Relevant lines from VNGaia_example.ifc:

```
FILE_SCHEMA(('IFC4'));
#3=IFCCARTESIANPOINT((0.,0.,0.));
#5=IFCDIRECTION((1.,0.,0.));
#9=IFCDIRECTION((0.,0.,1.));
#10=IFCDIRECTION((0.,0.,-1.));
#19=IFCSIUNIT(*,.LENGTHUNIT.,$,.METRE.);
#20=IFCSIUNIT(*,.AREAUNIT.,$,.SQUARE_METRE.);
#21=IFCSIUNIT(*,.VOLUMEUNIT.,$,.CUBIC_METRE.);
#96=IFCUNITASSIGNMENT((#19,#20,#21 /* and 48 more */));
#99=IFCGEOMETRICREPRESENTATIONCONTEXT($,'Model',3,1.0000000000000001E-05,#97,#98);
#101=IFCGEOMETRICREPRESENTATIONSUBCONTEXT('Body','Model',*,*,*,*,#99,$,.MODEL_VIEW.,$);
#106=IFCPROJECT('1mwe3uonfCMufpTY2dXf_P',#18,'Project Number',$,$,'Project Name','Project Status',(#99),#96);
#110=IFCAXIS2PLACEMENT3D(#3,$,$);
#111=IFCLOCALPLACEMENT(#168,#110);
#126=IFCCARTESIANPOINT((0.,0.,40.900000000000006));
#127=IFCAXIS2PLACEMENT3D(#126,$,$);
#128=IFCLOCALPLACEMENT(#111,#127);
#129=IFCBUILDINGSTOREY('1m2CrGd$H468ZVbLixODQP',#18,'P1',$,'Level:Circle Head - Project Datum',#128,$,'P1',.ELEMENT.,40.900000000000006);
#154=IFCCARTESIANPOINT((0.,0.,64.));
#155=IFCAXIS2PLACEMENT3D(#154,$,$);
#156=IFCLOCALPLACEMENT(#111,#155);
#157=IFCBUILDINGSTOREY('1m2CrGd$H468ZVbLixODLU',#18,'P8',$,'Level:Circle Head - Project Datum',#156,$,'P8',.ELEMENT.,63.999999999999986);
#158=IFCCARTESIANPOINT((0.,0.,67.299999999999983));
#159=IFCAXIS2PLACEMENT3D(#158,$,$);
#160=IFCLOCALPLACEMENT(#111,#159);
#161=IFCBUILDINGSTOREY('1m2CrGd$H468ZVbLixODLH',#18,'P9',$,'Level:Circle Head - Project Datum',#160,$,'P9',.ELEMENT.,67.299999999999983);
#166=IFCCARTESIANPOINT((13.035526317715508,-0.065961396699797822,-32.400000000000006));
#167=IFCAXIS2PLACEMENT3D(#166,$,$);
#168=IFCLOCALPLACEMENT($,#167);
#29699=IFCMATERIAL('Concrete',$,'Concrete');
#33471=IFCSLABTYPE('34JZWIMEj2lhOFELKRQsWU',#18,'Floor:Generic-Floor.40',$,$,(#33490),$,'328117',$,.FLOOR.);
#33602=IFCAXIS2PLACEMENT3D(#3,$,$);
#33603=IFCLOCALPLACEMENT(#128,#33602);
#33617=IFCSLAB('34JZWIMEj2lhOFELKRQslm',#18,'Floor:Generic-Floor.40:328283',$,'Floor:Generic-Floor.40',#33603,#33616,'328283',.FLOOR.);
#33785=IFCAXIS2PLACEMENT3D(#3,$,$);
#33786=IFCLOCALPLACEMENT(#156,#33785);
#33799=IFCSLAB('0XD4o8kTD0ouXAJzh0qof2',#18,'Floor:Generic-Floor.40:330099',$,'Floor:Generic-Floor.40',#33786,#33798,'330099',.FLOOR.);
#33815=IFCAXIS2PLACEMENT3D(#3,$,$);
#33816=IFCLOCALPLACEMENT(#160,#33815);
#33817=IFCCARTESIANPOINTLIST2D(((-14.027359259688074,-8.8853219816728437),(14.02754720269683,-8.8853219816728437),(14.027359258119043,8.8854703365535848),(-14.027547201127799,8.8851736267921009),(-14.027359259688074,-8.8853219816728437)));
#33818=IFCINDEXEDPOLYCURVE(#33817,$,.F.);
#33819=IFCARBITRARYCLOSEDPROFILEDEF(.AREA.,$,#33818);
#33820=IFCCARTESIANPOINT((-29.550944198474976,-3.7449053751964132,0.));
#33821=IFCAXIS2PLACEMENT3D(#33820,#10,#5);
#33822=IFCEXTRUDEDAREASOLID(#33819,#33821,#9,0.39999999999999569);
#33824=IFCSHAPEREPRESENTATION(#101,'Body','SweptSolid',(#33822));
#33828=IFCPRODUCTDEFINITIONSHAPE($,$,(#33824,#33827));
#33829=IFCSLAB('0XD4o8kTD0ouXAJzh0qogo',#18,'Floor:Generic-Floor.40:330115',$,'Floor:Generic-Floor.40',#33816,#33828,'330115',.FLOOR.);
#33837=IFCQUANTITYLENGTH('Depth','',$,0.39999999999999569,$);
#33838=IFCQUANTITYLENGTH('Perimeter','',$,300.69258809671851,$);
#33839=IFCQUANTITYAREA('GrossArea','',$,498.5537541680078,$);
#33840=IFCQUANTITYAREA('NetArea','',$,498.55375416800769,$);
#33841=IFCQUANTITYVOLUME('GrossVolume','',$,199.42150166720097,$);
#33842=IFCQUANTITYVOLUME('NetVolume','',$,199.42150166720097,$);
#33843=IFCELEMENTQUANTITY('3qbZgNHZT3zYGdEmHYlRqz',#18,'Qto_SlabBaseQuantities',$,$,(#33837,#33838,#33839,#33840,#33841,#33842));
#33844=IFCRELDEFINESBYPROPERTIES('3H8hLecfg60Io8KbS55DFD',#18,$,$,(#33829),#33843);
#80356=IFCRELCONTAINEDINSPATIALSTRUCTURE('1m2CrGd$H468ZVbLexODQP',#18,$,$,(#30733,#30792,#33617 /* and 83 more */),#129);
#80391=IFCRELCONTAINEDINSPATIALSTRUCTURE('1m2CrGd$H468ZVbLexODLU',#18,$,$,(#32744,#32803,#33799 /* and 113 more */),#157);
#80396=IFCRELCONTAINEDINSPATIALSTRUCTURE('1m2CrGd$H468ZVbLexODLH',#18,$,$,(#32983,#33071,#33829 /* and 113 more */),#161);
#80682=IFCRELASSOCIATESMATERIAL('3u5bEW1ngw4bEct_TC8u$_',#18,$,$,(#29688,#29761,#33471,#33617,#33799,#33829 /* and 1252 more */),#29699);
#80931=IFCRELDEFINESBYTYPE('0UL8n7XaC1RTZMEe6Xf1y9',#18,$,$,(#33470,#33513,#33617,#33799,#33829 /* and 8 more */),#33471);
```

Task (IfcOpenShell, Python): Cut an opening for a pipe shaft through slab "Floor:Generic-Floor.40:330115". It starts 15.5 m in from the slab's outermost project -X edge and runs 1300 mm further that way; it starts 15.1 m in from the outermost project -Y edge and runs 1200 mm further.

```python
import numpy as np
import ifcopenshell
import ifcopenshell.api.feature
import ifcopenshell.api.geometry
import ifcopenshell.api.pset
import ifcopenshell.api.root
import ifcopenshell.geom
import ifcopenshell.util.element
import ifcopenshell.util.placement
import ifcopenshell.util.representation
import ifcopenshell.util.shape
import ifcopenshell.util.unit

model = ifcopenshell.open("VNGaia_example.ifc")
unit_scale = ifcopenshell.util.unit.calculate_unit_scale(model)
area_scale = ifcopenshell.util.unit.calculate_unit_scale(model, "AREAUNIT")
volume_scale = ifcopenshell.util.unit.calculate_unit_scale(model, "VOLUMEUNIT")
settings = ifcopenshell.geom.settings()


def volume(element):
    """Net volume in cubic metres, openings subtracted."""
    shape = ifcopenshell.geom.create_shape(settings, element)
    return ifcopenshell.util.shape.get_volume(shape.geometry)


slab = model.by_guid("0XD4o8kTD0ouXAJzh0qogo")
before = volume(slab)

# Extent in the slab's own axes, in metres. The edges named are its -X and -Y sides.
slab_shape = ifcopenshell.geom.create_shape(settings, slab)
vertices = ifcopenshell.util.shape.get_vertices(slab_shape.geometry)
x_min, y_min, bottom = vertices.min(axis=0)
top = vertices[:, 2].max()

opening = ifcopenshell.api.root.create_entity(model, ifc_class="IfcOpeningElement", name="Pipe shaft opening", predefined_type="OPENING")
context = ifcopenshell.util.representation.get_context(model, "Model", "Body", "MODEL_VIEW")
width, depth = 1.3, 1.2
outline = [(0.0, 0.0), (width, 0.0), (width, depth), (0.0, depth), (0.0, 0.0)]
# Overshoot both faces by 50 mm so the cut is clean.
shape = ifcopenshell.api.geometry.add_slab_representation(
    model, context=context, depth=top - bottom + 0.1, polyline=outline
)
ifcopenshell.api.geometry.assign_representation(model, product=opening, representation=shape)

matrix = ifcopenshell.util.placement.get_local_placement(slab.ObjectPlacement)
matrix[:, 3] = matrix @ np.append(np.array([x_min + 15.5, y_min + 15.1, bottom - 0.05]) / unit_scale, 1.0)
ifcopenshell.api.geometry.edit_object_placement(model, product=opening, matrix=matrix, is_si=False)
ifcopenshell.api.feature.add_feature(model, feature=opening, element=slab)

after = volume(slab)

# Update the slab's stored quantities.
qto = model.by_id(ifcopenshell.util.element.get_pset(slab, "Qto_SlabBaseQuantities", should_inherit=False)["id"])
ifcopenshell.api.pset.edit_qto(model, qto=qto, properties={
    "NetArea": after / (top - bottom) / area_scale,
    "NetVolume": after / volume_scale,
})

print(f"slab volume {before:.3f} -> {after:.3f} m3")

model.write("VNGaia_example_rev.ifc")
```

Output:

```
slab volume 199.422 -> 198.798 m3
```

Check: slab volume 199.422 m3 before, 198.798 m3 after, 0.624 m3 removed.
